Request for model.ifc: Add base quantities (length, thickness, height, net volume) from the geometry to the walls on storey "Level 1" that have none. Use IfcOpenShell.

First a look at what the model holds.

```python
import ifcopenshell
import ifcopenshell.util.element
import ifcopenshell.util.unit

model = ifcopenshell.open("model.ifc")
print(model.schema)
for unit_type in ("LENGTHUNIT", "AREAUNIT", "VOLUMEUNIT"):
    print(unit_type, ifcopenshell.util.unit.calculate_unit_scale(model, unit_type))
storey = next(s for s in model.by_type("IfcBuildingStorey") if s.Name == "Level 1")
walls = [e for e in ifcopenshell.util.element.get_decomposition(storey) if e.is_a("IfcWall")]
for e in sorted(walls, key=lambda e: e.id()):
    print(e.id(), e.is_a(), e.Name, list(ifcopenshell.util.element.get_psets(e, qtos_only=True)), sep=" | ")
```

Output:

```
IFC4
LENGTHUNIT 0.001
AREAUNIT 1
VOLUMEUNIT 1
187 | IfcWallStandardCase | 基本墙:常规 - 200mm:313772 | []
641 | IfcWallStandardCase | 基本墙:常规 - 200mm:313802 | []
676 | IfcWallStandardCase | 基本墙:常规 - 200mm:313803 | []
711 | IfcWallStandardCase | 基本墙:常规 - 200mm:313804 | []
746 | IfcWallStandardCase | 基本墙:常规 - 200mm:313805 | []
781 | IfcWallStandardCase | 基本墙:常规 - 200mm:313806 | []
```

```python
import ifcopenshell
import ifcopenshell.api.pset
import ifcopenshell.geom
import ifcopenshell.util.element
import ifcopenshell.util.shape
import ifcopenshell.util.unit

model = ifcopenshell.open("model.ifc")
unit_scale = ifcopenshell.util.unit.calculate_unit_scale(model)
volume_scale = ifcopenshell.util.unit.calculate_unit_scale(model, "VOLUMEUNIT")
settings = ifcopenshell.geom.settings()

storey = next(s for s in model.by_type("IfcBuildingStorey") if s.Name == "Level 1")
walls = [e for e in ifcopenshell.util.element.get_decomposition(storey) if e.is_a("IfcWall")]

for e in sorted(walls, key=lambda e: e.id()):
    if ifcopenshell.util.element.get_psets(e, qtos_only=True, should_inherit=False):
        continue
    # Geometry comes back in metres, in the element's own axes.
    shape = ifcopenshell.geom.create_shape(settings, e)
    values = {
        "Length": ifcopenshell.util.shape.get_x(shape.geometry) / unit_scale,
        "Width": ifcopenshell.util.shape.get_y(shape.geometry) / unit_scale,
        "Height": ifcopenshell.util.shape.get_z(shape.geometry) / unit_scale,
        "NetVolume": ifcopenshell.util.shape.get_volume(shape.geometry) / volume_scale,
    }
    qto = ifcopenshell.api.pset.add_qto(model, product=e, name="Qto_WallBaseQuantities")
    ifcopenshell.api.pset.edit_qto(model, qto=qto, properties=values)
    print(e.id(), {k: round(v, 3) for k, v in values.items()})

model.write("model_updated.ifc")
```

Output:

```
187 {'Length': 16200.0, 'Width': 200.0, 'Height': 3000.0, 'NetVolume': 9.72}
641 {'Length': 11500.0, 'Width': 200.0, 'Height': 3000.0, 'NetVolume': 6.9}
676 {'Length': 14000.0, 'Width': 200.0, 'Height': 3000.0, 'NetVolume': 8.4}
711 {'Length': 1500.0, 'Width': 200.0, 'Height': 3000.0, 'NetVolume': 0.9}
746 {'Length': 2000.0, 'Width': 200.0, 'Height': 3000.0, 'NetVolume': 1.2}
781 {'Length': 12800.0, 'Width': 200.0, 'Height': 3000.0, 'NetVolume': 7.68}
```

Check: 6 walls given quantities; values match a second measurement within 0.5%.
